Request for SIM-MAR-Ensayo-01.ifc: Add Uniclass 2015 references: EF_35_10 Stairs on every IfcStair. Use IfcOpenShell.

First a look at what the model holds.

```python
import ifcopenshell

model = ifcopenshell.open("SIM-MAR-Ensayo-01.ifc")
print(model.schema)
print("classifications:", [c.Name for c in model.by_type("IfcClassification")])
for ifc_class in ("IfcDoor", "IfcRoof", "IfcStair", "IfcWall", "IfcWindow"):
    print(ifc_class, len(model.by_type(ifc_class)))
```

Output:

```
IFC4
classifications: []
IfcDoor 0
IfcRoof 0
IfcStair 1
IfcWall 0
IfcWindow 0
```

```python
import ifcopenshell
import ifcopenshell.api.classification

model = ifcopenshell.open("SIM-MAR-Ensayo-01.ifc")

system = ifcopenshell.api.classification.add_classification(model, classification="Uniclass 2015")

codes = {
    "IfcStair": ("EF_35_10", "Stairs"),
}
for ifc_class, (code, name) in codes.items():
    products = model.by_type(ifc_class)
    ifcopenshell.api.classification.add_reference(
        model, products=products, classification=system, identification=code, name=name
    )
    print(code, len(products))

model.write("SIM-MAR-Ensayo-01-out.ifc")
```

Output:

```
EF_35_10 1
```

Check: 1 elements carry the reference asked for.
